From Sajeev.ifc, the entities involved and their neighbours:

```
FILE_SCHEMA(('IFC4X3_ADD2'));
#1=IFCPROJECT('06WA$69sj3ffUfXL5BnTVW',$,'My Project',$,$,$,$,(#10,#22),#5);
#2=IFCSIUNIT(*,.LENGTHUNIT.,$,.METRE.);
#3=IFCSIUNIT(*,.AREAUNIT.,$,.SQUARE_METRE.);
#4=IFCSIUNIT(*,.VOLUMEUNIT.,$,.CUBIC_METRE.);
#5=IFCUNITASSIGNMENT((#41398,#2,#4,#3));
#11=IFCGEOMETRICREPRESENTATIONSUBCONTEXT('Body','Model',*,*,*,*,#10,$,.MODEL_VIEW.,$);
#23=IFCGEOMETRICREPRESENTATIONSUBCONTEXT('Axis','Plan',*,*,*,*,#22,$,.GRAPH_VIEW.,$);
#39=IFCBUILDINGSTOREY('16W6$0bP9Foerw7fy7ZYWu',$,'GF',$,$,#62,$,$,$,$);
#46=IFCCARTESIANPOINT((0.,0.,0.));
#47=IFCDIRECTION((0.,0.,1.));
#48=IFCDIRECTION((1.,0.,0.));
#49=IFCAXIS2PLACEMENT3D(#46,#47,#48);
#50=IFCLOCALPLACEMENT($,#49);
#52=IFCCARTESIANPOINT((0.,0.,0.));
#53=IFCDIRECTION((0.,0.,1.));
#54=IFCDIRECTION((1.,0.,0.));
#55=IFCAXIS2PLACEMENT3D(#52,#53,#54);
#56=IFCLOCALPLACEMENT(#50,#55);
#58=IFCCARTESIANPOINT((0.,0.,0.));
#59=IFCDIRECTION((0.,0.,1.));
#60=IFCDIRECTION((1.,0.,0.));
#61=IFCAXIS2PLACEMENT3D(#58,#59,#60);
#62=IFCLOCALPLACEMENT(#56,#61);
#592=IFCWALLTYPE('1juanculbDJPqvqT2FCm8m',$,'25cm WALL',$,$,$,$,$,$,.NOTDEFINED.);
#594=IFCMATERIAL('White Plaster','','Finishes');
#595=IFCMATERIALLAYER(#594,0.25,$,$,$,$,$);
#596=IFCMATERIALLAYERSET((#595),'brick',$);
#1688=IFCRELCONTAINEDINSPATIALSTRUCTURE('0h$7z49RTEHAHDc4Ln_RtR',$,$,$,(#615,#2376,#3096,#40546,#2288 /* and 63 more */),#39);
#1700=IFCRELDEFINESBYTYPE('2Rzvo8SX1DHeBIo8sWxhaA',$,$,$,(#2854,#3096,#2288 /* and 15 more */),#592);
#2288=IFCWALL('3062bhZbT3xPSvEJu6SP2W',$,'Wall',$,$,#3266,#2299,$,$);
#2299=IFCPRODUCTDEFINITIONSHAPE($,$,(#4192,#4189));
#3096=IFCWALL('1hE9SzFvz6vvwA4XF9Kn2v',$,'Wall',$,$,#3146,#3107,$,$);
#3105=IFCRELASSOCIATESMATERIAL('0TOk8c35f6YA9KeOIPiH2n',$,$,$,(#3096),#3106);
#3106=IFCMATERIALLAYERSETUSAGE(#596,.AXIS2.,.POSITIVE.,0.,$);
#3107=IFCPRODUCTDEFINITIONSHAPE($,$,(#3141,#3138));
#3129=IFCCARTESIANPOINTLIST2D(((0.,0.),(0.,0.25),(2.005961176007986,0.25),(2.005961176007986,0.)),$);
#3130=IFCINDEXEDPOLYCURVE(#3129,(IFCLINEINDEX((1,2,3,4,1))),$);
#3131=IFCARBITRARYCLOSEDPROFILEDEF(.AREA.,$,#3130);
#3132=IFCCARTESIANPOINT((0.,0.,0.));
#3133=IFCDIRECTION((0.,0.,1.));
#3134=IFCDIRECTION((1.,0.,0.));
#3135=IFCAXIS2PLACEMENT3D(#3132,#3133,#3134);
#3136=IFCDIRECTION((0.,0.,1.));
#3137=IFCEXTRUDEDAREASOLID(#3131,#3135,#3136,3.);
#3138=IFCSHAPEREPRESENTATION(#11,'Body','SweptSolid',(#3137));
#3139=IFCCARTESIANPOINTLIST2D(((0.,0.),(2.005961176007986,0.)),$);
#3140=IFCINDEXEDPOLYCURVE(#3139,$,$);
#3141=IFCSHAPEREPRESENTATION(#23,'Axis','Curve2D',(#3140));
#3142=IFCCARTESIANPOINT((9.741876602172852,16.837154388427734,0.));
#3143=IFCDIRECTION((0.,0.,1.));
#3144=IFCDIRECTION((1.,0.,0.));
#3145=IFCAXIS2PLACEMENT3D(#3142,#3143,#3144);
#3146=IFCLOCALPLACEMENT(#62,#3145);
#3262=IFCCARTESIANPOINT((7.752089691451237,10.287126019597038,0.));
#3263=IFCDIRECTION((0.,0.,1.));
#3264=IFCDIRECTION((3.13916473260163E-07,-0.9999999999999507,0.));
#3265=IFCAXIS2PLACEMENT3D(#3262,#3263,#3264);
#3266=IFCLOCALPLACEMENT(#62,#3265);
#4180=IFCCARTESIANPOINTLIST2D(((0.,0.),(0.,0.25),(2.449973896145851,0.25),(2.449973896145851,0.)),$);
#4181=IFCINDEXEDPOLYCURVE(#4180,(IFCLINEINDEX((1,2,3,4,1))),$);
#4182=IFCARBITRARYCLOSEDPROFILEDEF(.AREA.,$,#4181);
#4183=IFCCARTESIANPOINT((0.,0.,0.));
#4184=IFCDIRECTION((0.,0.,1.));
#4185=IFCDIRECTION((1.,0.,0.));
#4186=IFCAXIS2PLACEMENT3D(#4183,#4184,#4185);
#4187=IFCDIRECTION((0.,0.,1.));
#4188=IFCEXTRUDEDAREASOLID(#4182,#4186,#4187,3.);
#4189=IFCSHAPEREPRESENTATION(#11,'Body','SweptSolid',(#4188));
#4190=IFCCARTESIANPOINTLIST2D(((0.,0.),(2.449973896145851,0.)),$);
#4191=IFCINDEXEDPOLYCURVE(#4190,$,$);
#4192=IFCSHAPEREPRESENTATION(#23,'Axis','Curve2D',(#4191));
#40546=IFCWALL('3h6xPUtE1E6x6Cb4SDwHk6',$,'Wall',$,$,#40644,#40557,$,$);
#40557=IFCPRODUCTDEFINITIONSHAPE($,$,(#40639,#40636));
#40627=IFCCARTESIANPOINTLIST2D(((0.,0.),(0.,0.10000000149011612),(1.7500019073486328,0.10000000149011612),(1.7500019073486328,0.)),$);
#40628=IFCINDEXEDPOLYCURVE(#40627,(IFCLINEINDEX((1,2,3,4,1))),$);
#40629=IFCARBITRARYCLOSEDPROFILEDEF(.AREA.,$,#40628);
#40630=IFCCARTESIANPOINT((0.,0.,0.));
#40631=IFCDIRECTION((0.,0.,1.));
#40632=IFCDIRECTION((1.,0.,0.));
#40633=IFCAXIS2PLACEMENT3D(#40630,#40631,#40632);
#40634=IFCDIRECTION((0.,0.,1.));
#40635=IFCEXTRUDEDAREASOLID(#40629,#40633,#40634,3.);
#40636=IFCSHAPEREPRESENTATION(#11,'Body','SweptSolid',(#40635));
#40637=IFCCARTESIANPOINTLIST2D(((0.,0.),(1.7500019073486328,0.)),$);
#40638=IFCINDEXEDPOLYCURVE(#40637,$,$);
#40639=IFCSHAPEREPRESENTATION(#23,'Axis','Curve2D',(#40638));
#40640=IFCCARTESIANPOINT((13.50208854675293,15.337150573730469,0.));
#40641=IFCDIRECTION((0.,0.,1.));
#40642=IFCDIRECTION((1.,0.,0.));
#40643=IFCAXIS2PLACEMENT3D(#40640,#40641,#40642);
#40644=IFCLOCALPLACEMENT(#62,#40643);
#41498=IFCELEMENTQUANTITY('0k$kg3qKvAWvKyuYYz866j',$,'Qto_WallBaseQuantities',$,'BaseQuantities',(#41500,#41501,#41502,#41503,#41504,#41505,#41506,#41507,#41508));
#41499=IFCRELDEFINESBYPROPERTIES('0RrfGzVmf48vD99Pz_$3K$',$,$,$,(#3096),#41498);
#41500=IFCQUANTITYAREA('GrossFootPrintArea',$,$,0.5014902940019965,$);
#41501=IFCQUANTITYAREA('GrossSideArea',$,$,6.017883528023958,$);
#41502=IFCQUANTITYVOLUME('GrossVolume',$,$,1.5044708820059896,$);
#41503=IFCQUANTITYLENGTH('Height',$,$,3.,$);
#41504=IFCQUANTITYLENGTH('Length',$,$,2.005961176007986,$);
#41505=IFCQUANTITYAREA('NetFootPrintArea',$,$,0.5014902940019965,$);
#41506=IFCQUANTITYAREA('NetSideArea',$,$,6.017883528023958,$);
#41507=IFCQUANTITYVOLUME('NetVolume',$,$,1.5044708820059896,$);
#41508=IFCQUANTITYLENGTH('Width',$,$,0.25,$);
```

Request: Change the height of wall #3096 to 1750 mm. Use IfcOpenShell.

```python
import ifcopenshell
import ifcopenshell.api.pset
import ifcopenshell.geom
import ifcopenshell.util.element
import ifcopenshell.util.representation
import ifcopenshell.util.shape
import ifcopenshell.util.unit

model = ifcopenshell.open("Sajeev.ifc")
unit_scale = ifcopenshell.util.unit.calculate_unit_scale(model)
area_scale = ifcopenshell.util.unit.calculate_unit_scale(model, "AREAUNIT")
volume_scale = ifcopenshell.util.unit.calculate_unit_scale(model, "VOLUMEUNIT")
settings = ifcopenshell.geom.settings()


def volume(element):
    """Net volume in cubic metres, openings subtracted."""
    shape = ifcopenshell.geom.create_shape(settings, element)
    return ifcopenshell.util.shape.get_volume(shape.geometry)


wall = model.by_guid("1hE9SzFvz6vvwA4XF9Kn2v")
before = volume(wall)

body = ifcopenshell.util.representation.get_representation(wall, "Model", "Body")
solid = body.Items[0]
old_height = solid.Depth
solid.Depth = 1.75
after = volume(wall)
thickness = 0.25  # wall thickness in metres

# Update the stored height, areas and volumes.
qto = model.by_id(ifcopenshell.util.element.get_pset(wall, "Qto_WallBaseQuantities", should_inherit=False)["id"])
ifcopenshell.api.pset.edit_qto(model, qto=qto, properties={
    "GrossSideArea": ifcopenshell.util.element.get_pset(wall, "Qto_WallBaseQuantities", "GrossSideArea") * solid.Depth / old_height,
    "GrossVolume": ifcopenshell.util.element.get_pset(wall, "Qto_WallBaseQuantities", "GrossVolume") * solid.Depth / old_height,
    "Height": solid.Depth,
    "NetSideArea": after / thickness / area_scale,
    "NetVolume": after / volume_scale,
})

print(f"height {old_height:g} -> {solid.Depth:g}, volume {before:.3f} -> {after:.3f} m3")

model.write("Sajeev-out.ifc")
```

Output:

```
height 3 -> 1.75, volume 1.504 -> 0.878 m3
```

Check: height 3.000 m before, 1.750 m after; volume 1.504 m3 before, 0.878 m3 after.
